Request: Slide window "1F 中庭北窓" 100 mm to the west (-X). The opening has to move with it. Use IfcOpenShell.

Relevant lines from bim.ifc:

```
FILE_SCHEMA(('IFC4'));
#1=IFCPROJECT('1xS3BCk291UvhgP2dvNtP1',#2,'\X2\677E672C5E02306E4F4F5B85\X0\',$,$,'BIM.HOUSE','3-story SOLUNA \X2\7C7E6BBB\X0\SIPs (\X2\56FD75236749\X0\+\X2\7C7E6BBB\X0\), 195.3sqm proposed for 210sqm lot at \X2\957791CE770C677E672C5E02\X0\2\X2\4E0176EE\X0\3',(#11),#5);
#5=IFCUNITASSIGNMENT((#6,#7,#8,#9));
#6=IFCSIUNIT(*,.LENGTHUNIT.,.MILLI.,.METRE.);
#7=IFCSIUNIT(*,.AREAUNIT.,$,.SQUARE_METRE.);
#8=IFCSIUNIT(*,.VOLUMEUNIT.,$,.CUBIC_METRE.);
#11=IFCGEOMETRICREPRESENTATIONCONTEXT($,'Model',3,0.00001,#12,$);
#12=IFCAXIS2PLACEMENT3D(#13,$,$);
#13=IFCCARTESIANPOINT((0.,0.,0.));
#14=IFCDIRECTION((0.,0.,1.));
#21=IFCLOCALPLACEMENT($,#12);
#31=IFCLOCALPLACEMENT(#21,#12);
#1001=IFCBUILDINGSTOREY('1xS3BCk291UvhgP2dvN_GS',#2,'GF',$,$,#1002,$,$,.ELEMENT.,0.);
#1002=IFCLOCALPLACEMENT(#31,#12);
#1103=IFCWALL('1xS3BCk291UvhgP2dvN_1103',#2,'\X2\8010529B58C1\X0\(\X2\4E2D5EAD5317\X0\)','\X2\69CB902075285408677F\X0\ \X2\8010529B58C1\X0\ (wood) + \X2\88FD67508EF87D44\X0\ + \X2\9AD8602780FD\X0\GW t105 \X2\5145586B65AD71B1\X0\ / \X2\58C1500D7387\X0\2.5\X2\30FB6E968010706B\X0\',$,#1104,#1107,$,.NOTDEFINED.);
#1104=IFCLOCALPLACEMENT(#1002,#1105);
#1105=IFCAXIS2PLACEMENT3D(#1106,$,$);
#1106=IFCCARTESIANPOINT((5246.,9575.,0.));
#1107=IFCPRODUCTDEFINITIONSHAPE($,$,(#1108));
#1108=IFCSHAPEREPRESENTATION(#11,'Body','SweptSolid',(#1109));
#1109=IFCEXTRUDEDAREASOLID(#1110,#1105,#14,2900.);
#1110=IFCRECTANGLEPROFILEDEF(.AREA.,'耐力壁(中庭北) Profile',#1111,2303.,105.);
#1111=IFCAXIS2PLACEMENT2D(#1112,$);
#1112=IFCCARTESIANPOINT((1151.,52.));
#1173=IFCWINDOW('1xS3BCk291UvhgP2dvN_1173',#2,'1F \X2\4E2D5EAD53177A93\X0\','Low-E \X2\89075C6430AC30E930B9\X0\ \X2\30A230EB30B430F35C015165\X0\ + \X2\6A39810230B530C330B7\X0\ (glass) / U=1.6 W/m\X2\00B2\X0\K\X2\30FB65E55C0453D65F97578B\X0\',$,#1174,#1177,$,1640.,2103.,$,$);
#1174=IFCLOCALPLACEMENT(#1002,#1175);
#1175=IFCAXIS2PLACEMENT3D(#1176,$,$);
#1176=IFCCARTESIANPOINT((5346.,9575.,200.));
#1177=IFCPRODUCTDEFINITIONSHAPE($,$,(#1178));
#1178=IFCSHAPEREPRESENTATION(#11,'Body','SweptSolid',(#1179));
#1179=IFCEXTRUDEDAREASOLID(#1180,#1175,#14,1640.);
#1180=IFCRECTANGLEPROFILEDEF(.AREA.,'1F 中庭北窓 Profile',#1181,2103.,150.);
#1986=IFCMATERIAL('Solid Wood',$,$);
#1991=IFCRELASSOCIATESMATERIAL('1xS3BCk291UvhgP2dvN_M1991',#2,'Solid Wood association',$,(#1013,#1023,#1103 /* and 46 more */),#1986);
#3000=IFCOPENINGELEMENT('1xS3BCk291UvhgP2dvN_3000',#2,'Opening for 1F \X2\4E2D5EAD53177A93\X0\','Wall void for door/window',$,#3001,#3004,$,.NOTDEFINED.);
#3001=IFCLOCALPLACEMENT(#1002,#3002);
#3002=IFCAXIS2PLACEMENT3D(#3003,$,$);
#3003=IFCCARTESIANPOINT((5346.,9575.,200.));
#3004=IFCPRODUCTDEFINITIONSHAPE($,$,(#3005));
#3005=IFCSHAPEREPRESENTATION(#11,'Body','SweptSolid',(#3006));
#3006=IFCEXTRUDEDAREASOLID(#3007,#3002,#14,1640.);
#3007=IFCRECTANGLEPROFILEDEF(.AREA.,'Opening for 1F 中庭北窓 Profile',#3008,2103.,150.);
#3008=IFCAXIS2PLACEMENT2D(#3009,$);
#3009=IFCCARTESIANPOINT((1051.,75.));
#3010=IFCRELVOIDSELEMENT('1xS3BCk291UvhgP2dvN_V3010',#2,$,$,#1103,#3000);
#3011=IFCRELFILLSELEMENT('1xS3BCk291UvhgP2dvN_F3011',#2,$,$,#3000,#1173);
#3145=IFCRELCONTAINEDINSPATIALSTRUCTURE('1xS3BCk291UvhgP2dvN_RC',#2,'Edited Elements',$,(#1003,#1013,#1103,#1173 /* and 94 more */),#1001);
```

```python
import ifcopenshell
import ifcopenshell.api.geometry
import ifcopenshell.util.placement
import ifcopenshell.util.unit

model = ifcopenshell.open("bim.ifc")
unit_scale = ifcopenshell.util.unit.calculate_unit_scale(model)

window = model.by_guid("1xS3BCk291UvhgP2dvN_1173")
opening = window.FillsVoids[0].RelatingOpeningElement
wall = opening.VoidsElements[0].RelatingBuildingElement

wall_matrix = ifcopenshell.util.placement.get_local_placement(wall.ObjectPlacement)
shift = wall_matrix[:3, 0] * -0.1 / unit_scale
before = ifcopenshell.util.placement.get_local_placement(window.ObjectPlacement)[:3, 3].copy()

# The window is not placed relative to its opening, so move both.
for product in (opening, window):
    matrix = ifcopenshell.util.placement.get_local_placement(product.ObjectPlacement)
    matrix[:3, 3] += shift
    ifcopenshell.api.geometry.edit_object_placement(model, product=product, matrix=matrix, is_si=False)

after = ifcopenshell.util.placement.get_local_placement(window.ObjectPlacement)[:3, 3]
print("window moved by", (after - before).round(3) + 0.0)

model.write("bim_updated.ifc")
```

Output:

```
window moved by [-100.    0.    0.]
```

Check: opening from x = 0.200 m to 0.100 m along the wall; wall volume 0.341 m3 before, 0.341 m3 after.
